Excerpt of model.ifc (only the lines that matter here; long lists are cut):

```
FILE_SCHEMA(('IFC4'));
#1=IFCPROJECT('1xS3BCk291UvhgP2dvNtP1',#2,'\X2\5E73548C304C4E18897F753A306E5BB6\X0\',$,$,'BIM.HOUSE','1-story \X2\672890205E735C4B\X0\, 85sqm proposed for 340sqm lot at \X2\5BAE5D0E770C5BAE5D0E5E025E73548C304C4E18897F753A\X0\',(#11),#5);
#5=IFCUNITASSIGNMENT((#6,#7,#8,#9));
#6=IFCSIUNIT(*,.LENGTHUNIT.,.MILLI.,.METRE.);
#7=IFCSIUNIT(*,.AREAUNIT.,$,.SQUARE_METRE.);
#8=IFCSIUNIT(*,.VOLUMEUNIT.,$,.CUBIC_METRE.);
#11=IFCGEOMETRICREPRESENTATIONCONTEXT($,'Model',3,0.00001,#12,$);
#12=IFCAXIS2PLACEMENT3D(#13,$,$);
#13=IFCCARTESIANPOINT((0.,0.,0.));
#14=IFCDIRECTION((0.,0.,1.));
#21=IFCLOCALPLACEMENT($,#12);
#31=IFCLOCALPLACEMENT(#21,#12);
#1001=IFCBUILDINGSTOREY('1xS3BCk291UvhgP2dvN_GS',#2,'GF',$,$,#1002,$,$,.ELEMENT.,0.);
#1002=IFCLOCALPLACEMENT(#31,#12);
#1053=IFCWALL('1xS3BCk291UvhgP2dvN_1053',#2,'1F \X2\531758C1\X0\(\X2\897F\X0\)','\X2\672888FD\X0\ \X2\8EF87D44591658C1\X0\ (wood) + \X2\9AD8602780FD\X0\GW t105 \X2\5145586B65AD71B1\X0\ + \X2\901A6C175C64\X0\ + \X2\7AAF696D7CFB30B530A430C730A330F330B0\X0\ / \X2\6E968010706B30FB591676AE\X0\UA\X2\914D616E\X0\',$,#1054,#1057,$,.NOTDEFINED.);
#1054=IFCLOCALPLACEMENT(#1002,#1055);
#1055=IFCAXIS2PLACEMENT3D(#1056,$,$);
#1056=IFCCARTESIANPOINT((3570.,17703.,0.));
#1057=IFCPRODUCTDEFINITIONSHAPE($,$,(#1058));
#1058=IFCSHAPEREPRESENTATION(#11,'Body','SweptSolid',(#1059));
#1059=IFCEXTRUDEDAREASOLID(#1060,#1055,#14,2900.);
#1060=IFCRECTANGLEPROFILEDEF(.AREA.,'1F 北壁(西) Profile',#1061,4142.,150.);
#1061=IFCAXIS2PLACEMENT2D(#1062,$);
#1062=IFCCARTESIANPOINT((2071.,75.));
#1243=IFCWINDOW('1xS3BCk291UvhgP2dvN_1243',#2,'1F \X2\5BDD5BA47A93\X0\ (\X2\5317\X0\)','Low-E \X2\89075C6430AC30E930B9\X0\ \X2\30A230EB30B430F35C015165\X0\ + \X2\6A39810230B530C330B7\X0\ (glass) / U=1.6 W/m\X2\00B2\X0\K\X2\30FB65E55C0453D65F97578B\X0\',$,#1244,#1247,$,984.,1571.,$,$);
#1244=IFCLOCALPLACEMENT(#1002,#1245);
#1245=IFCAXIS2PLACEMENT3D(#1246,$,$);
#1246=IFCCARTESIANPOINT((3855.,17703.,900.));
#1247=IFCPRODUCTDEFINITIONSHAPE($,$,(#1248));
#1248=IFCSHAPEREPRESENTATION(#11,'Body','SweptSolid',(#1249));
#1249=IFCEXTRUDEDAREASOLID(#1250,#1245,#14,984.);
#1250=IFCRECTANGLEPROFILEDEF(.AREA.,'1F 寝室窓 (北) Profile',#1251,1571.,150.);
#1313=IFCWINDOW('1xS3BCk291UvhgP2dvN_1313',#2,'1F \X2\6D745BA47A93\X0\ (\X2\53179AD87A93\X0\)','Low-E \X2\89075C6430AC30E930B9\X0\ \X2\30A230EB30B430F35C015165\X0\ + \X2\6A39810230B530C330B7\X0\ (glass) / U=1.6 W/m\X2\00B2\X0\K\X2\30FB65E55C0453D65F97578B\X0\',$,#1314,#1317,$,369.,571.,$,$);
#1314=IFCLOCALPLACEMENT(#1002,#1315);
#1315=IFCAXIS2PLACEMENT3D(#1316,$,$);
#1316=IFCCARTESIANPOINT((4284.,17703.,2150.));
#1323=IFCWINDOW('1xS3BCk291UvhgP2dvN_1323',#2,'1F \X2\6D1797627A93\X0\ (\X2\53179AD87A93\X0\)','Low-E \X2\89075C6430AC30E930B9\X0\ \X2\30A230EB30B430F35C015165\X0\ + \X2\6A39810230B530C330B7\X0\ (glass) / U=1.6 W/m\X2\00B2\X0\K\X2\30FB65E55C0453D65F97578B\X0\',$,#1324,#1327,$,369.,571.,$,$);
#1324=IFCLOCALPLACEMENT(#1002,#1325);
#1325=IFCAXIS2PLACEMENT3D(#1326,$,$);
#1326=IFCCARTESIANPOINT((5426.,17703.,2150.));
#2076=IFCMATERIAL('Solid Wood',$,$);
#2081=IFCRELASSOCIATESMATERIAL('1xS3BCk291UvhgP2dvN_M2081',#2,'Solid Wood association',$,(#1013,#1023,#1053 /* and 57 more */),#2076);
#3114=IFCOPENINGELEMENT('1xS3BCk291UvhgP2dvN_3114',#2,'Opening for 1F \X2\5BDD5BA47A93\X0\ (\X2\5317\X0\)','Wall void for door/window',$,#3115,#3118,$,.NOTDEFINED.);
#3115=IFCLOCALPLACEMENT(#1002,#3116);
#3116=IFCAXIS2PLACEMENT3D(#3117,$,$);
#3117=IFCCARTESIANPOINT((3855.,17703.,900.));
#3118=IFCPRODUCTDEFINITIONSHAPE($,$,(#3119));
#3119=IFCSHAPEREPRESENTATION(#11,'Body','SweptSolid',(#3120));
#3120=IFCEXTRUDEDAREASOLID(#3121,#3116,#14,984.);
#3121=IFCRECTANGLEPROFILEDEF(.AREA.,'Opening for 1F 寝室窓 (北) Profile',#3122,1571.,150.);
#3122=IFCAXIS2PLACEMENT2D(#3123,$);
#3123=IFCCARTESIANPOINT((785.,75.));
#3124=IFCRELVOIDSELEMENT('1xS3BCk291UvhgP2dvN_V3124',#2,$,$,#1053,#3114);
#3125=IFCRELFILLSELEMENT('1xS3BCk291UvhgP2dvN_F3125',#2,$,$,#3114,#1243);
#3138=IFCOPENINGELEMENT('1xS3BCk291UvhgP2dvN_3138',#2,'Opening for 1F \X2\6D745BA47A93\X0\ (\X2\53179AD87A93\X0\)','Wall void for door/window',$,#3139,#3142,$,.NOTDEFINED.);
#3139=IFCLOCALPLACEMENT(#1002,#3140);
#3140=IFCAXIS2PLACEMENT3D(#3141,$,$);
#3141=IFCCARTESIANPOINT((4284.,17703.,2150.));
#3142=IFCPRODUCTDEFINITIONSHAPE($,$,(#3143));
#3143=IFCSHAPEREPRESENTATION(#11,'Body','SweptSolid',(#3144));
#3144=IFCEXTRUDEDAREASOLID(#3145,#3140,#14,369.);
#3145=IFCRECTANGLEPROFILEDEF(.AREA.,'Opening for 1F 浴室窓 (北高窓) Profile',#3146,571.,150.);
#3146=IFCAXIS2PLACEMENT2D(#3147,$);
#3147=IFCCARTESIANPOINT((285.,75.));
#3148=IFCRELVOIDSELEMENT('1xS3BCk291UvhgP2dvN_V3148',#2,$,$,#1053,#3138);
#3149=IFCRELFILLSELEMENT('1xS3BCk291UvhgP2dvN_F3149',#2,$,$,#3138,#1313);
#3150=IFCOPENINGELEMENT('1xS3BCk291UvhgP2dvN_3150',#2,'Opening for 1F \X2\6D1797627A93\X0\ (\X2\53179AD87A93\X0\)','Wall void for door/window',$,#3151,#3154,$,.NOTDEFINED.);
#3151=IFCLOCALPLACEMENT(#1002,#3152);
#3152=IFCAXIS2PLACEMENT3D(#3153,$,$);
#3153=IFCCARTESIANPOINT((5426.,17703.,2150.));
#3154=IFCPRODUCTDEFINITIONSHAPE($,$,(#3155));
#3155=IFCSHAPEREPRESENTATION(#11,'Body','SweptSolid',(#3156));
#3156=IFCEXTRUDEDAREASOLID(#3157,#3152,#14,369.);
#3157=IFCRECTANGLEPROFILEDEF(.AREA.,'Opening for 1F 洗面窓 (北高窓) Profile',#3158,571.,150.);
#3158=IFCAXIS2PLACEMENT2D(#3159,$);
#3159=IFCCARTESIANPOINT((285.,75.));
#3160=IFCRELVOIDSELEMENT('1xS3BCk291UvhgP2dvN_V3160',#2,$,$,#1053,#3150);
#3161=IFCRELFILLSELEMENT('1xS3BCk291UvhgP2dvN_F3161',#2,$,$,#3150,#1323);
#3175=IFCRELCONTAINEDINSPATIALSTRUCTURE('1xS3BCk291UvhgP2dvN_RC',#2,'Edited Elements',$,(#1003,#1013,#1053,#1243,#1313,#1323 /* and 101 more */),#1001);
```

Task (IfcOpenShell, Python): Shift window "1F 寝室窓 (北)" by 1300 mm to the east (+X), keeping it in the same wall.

```python
import ifcopenshell
import ifcopenshell.api.geometry
import ifcopenshell.util.placement

model = ifcopenshell.open("model.ifc")

window = model.by_guid("1xS3BCk291UvhgP2dvN_1243")
opening = window.FillsVoids[0].RelatingOpeningElement
wall = opening.VoidsElements[0].RelatingBuildingElement

wall_matrix = ifcopenshell.util.placement.get_local_placement(wall.ObjectPlacement)
shift = wall_matrix[:3, 0] * 1300.0
before = ifcopenshell.util.placement.get_local_placement(window.ObjectPlacement)[:3, 3].copy()

# The window is not placed relative to its opening, so move both.
for product in (opening, window):
    matrix = ifcopenshell.util.placement.get_local_placement(product.ObjectPlacement)
    matrix[:3, 3] += shift
    ifcopenshell.api.geometry.edit_object_placement(model, product=product, matrix=matrix, is_si=False)

after = ifcopenshell.util.placement.get_local_placement(window.ObjectPlacement)[:3, 3]
print("window moved by", (after - before).round(3) + 0.0)

model.write("model_rev.ifc")
```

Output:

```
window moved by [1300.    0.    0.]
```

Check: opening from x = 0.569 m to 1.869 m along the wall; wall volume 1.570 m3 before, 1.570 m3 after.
